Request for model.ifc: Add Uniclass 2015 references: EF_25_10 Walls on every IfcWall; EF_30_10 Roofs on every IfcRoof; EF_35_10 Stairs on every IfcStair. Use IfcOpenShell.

First a look at what the model holds.

```python
import ifcopenshell

model = ifcopenshell.open("model.ifc")
print(model.schema)
print("classifications:", [c.Name for c in model.by_type("IfcClassification")])
for ifc_class in ("IfcDoor", "IfcRoof", "IfcStair", "IfcWall", "IfcWindow"):
    print(ifc_class, len(model.by_type(ifc_class)))
```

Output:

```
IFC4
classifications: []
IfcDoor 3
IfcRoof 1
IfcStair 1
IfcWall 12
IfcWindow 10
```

```python
import ifcopenshell
import ifcopenshell.api.classification

model = ifcopenshell.open("model.ifc")

system = ifcopenshell.api.classification.add_classification(model, classification="Uniclass 2015")

codes = {
    "IfcWall": ("EF_25_10", "Walls"),
    "IfcRoof": ("EF_30_10", "Roofs"),
    "IfcStair": ("EF_35_10", "Stairs"),
}
for ifc_class, (code, name) in codes.items():
    products = model.by_type(ifc_class)
    ifcopenshell.api.classification.add_reference(
        model, products=products, classification=system, identification=code, name=name
    )
    print(code, len(products))

model.write("model_v2.ifc")
```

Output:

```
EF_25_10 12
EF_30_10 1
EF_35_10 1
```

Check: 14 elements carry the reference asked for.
